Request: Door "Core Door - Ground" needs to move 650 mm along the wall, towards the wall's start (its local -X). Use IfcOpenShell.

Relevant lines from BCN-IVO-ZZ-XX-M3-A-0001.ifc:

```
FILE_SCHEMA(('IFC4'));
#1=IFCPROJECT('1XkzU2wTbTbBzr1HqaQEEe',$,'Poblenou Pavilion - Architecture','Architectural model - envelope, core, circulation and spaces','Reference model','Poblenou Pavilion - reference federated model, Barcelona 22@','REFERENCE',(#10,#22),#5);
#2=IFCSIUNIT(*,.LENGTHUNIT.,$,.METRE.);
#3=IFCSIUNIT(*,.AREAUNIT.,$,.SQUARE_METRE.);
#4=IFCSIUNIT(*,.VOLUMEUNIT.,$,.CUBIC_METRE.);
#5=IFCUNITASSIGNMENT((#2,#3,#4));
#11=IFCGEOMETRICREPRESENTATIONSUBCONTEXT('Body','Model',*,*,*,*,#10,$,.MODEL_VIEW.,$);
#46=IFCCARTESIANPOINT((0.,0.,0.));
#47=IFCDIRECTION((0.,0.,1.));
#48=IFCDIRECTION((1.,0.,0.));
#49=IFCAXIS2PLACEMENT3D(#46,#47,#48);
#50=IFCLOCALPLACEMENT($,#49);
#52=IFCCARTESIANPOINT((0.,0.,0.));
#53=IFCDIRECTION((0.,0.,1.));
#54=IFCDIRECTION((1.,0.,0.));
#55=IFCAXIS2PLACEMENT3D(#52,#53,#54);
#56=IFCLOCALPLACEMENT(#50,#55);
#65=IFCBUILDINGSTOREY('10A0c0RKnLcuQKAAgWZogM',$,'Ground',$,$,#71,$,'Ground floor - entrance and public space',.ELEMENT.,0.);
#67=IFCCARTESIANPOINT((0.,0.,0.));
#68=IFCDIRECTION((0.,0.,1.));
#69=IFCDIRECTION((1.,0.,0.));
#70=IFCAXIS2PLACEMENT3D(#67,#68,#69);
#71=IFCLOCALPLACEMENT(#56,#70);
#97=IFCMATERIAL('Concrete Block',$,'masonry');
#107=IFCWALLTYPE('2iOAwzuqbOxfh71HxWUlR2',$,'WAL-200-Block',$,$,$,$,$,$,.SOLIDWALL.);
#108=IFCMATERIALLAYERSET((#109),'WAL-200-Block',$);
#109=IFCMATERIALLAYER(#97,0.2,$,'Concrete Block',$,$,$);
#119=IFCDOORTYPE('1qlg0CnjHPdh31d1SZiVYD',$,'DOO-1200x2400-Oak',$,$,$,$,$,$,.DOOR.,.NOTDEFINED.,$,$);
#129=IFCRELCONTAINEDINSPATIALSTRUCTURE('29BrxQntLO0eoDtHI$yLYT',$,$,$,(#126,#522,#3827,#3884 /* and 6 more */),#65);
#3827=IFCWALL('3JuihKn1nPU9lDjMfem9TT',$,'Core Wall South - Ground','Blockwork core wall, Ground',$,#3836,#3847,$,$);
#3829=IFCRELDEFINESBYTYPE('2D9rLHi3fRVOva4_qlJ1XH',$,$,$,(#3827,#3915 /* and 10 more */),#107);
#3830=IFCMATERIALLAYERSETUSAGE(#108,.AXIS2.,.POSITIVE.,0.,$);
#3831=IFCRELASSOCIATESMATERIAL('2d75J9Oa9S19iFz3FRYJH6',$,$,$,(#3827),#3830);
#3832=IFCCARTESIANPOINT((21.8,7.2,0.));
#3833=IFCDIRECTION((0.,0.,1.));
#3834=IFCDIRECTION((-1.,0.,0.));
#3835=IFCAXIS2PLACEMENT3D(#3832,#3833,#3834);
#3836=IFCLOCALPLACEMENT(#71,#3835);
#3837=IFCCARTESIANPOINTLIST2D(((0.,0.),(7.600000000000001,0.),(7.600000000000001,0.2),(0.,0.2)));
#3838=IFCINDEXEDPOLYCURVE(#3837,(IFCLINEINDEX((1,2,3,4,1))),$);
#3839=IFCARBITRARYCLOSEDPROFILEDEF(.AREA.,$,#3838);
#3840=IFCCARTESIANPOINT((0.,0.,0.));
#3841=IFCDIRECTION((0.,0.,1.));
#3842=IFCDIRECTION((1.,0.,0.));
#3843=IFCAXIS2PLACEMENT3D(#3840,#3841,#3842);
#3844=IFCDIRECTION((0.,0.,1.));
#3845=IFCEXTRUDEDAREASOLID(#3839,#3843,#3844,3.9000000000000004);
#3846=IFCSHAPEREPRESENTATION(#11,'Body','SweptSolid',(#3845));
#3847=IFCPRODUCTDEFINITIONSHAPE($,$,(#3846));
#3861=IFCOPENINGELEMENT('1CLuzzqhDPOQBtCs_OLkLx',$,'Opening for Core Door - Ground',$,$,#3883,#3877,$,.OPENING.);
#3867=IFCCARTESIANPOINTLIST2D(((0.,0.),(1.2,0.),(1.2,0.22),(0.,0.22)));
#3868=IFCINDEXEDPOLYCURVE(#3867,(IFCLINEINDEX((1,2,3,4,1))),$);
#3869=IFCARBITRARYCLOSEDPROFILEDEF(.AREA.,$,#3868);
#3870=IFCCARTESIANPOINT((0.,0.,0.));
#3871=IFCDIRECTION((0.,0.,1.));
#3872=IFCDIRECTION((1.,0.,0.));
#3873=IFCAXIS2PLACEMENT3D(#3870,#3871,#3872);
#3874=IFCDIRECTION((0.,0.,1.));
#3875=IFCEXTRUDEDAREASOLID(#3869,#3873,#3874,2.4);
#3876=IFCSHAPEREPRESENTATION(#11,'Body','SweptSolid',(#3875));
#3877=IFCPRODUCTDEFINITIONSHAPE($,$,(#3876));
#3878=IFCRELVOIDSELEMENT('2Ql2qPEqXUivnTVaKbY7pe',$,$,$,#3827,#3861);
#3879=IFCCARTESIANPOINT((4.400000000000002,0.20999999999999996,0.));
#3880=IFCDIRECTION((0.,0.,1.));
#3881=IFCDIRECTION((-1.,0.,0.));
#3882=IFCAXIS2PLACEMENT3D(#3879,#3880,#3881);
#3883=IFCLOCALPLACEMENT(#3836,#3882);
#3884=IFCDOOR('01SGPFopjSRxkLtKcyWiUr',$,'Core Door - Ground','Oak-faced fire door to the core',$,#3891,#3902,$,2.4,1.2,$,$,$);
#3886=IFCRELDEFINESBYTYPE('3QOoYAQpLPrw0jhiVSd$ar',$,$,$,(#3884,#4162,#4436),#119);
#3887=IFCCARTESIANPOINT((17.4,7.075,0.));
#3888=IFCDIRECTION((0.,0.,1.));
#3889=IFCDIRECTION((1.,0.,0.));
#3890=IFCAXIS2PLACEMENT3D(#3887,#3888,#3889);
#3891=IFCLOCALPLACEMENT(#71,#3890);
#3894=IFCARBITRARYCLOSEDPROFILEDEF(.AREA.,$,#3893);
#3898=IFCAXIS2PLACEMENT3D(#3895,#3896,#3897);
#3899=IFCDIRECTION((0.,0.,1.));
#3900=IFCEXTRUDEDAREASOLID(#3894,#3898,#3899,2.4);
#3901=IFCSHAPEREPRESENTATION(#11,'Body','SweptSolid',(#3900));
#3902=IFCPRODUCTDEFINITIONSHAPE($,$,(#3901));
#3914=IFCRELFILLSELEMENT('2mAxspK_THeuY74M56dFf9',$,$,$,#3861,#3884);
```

```python
import ifcopenshell
import ifcopenshell.api.geometry
import ifcopenshell.util.placement

model = ifcopenshell.open("BCN-IVO-ZZ-XX-M3-A-0001.ifc")

door = model.by_guid("01SGPFopjSRxkLtKcyWiUr")
opening = door.FillsVoids[0].RelatingOpeningElement
wall = opening.VoidsElements[0].RelatingBuildingElement

wall_matrix = ifcopenshell.util.placement.get_local_placement(wall.ObjectPlacement)
shift = wall_matrix[:3, 0] * -0.65
before = ifcopenshell.util.placement.get_local_placement(door.ObjectPlacement)[:3, 3].copy()

# The door is not placed relative to its opening, so move both.
for product in (opening, door):
    matrix = ifcopenshell.util.placement.get_local_placement(product.ObjectPlacement)
    matrix[:3, 3] += shift
    ifcopenshell.api.geometry.edit_object_placement(model, product=product, matrix=matrix, is_si=False)

after = ifcopenshell.util.placement.get_local_placement(door.ObjectPlacement)[:3, 3]
print("door moved by", (after - before).round(3) + 0.0)

model.write("BCN-IVO-ZZ-XX-M3-A-0001-out.ifc")
```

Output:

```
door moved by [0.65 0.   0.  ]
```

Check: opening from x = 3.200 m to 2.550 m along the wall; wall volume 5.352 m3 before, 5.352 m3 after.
